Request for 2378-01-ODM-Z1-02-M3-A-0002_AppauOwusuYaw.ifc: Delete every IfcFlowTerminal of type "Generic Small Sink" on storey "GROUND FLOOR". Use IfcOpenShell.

First a look at what the model holds.

```python
import ifcopenshell
import ifcopenshell.util.element

model = ifcopenshell.open("2378-01-ODM-Z1-02-M3-A-0002_AppauOwusuYaw.ifc")
print(model.schema)
storey = next(s for s in model.by_type("IfcBuildingStorey") if s.Name == "GROUND FLOOR")
terminals = [e for e in ifcopenshell.util.element.get_decomposition(storey) if e.is_a("IfcFlowTerminal")]
seen = {}
for e in terminals:
    element_type = ifcopenshell.util.element.get_type(e)
    name = element_type.Name if element_type not in (None, e) else None
    seen[name] = seen.get(name, 0) + 1
for name, count in sorted(seen.items(), key=str):
    print(count, "x", name)
```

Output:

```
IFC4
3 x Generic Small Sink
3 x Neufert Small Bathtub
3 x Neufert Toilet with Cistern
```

```python
import ifcopenshell
import ifcopenshell.api.root
import ifcopenshell.util.element

model = ifcopenshell.open("2378-01-ODM-Z1-02-M3-A-0002_AppauOwusuYaw.ifc")

storey = next(s for s in model.by_type("IfcBuildingStorey") if s.Name == "GROUND FLOOR")
terminals = [e for e in ifcopenshell.util.element.get_decomposition(storey) if e.is_a("IfcFlowTerminal")]
targets = [e for e in terminals if (t := ifcopenshell.util.element.get_type(e)) not in (None, e) and t.Name == "Generic Small Sink"]

for e in targets:
    ifcopenshell.api.root.remove_product(model, product=e)
print(len(targets), "removed")

model.write("2378-01-ODM-Z1-02-M3-A-0002_AppauOwusuYaw_updated.ifc")
```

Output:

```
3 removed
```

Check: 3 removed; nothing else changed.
